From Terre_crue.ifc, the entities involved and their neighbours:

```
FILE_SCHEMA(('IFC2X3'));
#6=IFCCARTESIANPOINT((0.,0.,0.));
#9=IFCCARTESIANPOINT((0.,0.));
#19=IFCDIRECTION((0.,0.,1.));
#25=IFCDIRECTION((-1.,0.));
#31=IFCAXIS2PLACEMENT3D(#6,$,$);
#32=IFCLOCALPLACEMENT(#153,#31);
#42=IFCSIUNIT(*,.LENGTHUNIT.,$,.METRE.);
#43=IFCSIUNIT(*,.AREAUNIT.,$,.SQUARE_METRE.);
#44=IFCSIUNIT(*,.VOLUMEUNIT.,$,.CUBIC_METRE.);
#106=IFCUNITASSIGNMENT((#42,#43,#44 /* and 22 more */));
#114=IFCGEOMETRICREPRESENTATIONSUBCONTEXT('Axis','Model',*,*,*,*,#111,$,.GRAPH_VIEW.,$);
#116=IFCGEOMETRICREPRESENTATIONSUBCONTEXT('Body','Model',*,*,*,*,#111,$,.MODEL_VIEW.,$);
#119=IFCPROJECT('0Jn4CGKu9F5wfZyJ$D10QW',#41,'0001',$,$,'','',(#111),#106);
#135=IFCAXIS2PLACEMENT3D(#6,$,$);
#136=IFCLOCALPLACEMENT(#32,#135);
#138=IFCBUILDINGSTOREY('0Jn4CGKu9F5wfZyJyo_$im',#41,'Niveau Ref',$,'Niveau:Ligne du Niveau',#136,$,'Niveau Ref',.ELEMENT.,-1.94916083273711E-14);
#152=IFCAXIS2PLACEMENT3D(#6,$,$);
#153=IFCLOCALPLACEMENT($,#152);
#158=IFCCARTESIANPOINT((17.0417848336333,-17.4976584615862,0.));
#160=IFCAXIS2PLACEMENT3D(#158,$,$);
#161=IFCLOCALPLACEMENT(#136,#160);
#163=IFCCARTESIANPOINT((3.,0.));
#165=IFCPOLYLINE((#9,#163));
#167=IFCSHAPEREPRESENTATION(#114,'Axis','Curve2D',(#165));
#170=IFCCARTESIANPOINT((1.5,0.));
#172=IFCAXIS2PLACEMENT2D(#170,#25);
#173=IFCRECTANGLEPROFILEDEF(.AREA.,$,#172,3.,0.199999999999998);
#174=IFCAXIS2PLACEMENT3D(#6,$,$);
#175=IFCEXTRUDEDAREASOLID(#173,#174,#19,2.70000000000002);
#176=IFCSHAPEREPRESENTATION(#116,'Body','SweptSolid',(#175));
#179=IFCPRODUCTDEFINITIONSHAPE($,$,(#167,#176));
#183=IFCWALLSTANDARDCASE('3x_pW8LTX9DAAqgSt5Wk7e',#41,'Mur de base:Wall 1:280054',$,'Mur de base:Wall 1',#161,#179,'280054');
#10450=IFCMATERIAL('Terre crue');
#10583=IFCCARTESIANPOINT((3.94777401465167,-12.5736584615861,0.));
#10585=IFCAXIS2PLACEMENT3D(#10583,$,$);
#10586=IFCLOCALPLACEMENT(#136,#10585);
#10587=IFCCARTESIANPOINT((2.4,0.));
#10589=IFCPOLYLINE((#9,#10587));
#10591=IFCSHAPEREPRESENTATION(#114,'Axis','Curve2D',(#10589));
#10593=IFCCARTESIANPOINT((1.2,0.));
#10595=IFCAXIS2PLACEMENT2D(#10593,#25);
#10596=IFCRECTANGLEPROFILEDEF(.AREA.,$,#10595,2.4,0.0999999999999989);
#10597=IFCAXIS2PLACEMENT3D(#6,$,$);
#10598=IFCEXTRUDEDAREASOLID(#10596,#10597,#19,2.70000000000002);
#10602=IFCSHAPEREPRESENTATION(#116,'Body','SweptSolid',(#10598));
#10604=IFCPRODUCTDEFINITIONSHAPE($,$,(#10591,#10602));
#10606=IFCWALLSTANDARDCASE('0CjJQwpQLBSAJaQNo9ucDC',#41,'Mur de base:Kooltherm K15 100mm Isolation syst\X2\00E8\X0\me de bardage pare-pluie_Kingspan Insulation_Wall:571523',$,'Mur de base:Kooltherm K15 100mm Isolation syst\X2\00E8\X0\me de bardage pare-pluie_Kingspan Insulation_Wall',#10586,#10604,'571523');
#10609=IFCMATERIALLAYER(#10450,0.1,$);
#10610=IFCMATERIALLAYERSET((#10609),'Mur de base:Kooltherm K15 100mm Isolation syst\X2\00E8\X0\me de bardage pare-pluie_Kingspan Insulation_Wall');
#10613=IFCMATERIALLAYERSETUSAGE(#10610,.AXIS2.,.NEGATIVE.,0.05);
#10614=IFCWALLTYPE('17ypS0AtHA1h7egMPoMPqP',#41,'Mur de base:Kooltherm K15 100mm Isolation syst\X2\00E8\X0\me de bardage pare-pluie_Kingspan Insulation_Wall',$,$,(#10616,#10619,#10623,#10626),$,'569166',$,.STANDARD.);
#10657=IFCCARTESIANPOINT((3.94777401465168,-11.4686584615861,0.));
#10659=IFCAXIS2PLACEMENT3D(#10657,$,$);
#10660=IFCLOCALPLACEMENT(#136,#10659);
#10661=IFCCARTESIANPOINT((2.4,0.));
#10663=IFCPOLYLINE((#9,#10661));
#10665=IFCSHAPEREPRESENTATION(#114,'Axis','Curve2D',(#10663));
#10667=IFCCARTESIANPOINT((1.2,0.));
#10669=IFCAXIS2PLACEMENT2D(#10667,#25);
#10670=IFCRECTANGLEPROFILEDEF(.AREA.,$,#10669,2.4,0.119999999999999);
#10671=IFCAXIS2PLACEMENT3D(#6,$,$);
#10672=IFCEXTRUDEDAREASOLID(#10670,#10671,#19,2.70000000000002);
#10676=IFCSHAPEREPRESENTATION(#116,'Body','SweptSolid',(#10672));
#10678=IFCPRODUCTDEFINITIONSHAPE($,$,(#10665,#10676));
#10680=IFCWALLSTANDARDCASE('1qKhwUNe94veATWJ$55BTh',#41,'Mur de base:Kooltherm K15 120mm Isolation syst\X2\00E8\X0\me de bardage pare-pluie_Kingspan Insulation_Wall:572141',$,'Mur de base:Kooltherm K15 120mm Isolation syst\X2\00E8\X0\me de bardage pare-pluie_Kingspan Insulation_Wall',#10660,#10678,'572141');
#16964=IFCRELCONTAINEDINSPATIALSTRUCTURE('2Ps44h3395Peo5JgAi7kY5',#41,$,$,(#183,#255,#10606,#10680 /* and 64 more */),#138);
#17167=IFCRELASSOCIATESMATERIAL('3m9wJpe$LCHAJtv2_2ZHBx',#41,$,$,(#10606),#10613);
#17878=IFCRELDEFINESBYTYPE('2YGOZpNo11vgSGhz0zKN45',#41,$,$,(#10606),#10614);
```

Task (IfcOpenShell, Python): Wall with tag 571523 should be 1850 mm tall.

```python
import ifcopenshell
import ifcopenshell.geom
import ifcopenshell.util.representation
import ifcopenshell.util.shape
import ifcopenshell.util.unit

model = ifcopenshell.open("Terre_crue.ifc")
unit_scale = ifcopenshell.util.unit.calculate_unit_scale(model)
settings = ifcopenshell.geom.settings()


def volume(element):
    """Net volume in cubic metres, openings subtracted."""
    shape = ifcopenshell.geom.create_shape(settings, element)
    return ifcopenshell.util.shape.get_volume(shape.geometry)


wall = model.by_id(10606)
before = volume(wall)

body = ifcopenshell.util.representation.get_representation(wall, "Model", "Body")
solid = body.Items[0]
old_height = solid.Depth
solid.Depth = 1.85 / unit_scale
after = volume(wall)

print(f"height {old_height:g} -> {solid.Depth:g}, volume {before:.3f} -> {after:.3f} m3")

model.write("Terre_crue_updated.ifc")
```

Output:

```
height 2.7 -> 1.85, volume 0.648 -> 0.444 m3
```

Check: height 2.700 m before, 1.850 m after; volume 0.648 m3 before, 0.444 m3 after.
